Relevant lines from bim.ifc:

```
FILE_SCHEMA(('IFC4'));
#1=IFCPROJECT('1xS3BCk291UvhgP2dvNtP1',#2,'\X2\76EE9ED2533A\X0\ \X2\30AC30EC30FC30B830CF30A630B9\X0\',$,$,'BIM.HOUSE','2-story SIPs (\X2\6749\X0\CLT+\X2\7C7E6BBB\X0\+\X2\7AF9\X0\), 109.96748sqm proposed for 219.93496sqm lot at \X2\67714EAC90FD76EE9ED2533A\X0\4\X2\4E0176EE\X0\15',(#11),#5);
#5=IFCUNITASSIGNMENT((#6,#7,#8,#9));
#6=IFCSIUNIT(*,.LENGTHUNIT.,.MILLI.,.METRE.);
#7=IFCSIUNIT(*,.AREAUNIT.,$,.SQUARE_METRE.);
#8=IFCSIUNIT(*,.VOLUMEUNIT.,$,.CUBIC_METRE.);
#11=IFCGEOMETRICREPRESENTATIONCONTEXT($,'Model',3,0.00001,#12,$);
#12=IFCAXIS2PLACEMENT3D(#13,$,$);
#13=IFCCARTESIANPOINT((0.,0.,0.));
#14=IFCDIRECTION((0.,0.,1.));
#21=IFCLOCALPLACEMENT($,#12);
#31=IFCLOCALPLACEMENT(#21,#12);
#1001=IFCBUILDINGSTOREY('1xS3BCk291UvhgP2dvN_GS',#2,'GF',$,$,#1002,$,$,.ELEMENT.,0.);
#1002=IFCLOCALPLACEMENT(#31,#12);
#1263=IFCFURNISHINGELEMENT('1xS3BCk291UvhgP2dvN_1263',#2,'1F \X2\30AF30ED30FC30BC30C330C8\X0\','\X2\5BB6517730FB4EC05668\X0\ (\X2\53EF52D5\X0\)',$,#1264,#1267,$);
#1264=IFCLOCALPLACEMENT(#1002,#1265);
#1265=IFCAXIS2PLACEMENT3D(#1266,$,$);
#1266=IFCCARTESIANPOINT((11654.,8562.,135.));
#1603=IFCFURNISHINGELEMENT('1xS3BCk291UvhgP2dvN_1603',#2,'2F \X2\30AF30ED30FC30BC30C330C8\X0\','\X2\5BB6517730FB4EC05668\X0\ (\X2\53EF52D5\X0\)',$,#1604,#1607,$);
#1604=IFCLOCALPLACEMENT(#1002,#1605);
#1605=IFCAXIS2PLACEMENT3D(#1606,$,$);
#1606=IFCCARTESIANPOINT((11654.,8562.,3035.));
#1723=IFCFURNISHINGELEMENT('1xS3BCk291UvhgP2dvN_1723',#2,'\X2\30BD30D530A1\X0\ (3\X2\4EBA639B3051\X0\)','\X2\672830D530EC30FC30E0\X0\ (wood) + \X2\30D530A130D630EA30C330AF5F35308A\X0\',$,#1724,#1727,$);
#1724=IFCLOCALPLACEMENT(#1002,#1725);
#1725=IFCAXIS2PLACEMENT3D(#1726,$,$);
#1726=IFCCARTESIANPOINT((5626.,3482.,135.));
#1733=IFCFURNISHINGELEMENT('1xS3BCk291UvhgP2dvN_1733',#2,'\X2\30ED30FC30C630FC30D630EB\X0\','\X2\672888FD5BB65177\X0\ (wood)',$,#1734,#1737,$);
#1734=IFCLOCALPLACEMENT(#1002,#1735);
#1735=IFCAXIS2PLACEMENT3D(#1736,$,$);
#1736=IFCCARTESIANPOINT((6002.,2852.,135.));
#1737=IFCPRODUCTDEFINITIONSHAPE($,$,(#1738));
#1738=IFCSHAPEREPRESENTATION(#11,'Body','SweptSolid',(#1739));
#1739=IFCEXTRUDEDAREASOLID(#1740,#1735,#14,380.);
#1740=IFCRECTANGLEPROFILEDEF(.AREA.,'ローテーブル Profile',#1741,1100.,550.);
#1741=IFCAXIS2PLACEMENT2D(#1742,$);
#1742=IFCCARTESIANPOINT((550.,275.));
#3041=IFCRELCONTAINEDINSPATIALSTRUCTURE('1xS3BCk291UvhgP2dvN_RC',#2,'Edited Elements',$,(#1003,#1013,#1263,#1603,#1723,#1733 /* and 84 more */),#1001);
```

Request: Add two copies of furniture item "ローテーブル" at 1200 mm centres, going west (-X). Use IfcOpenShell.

```python
import numpy as np
import ifcopenshell
import ifcopenshell.api.geometry
import ifcopenshell.api.root
import ifcopenshell.util.element
import ifcopenshell.util.placement
import ifcopenshell.util.unit

model = ifcopenshell.open("bim.ifc")
unit_scale = ifcopenshell.util.unit.calculate_unit_scale(model)


def reuse_history(source, copy):
    """copy_class also copies each property set's owner history, people and application; keep the originals."""
    for rel in copy.IsDefinedBy:
        if rel.is_a("IfcRelDefinesByProperties") and (history := rel.RelatingPropertyDefinition.OwnerHistory):
            rel.RelatingPropertyDefinition.OwnerHistory = source.OwnerHistory
            ifcopenshell.util.element.remove_deep2(model, history)


source = model.by_id(1733)
base = ifcopenshell.util.placement.get_local_placement(source.ObjectPlacement)
step = np.array([-1.0, 0.0, 0.0]) * 1.2 / unit_scale

for i in range(1, 3):
    copy = ifcopenshell.api.root.copy_class(model, product=source)
    copy.Representation = ifcopenshell.util.element.copy_deep(
        model, source.Representation, exclude=["IfcGeometricRepresentationContext", "IfcRepresentationMap"]
    )
    reuse_history(source, copy)
    matrix = base.copy()
    matrix[:3, 3] += i * step
    print("added at", matrix[:3, 3].round(3) + 0.0)
    ifcopenshell.api.geometry.edit_object_placement(model, product=copy, matrix=matrix, is_si=False)

model.write("bim_updated.ifc")
```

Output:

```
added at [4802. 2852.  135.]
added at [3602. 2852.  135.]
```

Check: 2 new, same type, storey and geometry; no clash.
